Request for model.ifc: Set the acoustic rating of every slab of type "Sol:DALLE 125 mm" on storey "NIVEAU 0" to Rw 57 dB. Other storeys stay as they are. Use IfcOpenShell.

First a look at what the model holds.

```python
import ifcopenshell
import ifcopenshell.util.element

model = ifcopenshell.open("model.ifc")
print(model.schema)
storey = next(s for s in model.by_type("IfcBuildingStorey") if s.Name == "NIVEAU 0")
slabs = [e for e in ifcopenshell.util.element.get_decomposition(storey) if e.is_a("IfcSlab")]
seen = {}
for e in slabs:
    element_type = ifcopenshell.util.element.get_type(e)
    key = (element_type.Name if element_type != e and element_type else None, ifcopenshell.util.element.get_pset(e, "Pset_SlabCommon", "AcousticRating"))
    seen[key] = seen.get(key, 0) + 1
for (name, value), count in sorted(seen.items(), key=str):
    print(count, "x", name, "|", value)
```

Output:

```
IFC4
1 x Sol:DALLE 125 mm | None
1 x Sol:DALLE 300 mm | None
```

```python
import ifcopenshell
import ifcopenshell.api.pset
import ifcopenshell.util.element

model = ifcopenshell.open("model.ifc")

storey = next(s for s in model.by_type("IfcBuildingStorey") if s.Name == "NIVEAU 0")
slabs = [e for e in ifcopenshell.util.element.get_decomposition(storey) if e.is_a("IfcSlab")]

count = 0
for e in slabs:
    element_type = ifcopenshell.util.element.get_type(e)
    if element_type in (None, e) or element_type.Name != "Sol:DALLE 125 mm":
        continue
    # add_pset returns the element's existing set when there is one.
    pset = ifcopenshell.api.pset.add_pset(model, product=e, name="Pset_SlabCommon")
    ifcopenshell.api.pset.edit_pset(model, pset=pset, properties={"AcousticRating": "Rw 57 dB"})
    count += 1

print(count, "slabs updated")

model.write("model_v2.ifc")
```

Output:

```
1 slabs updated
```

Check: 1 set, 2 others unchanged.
